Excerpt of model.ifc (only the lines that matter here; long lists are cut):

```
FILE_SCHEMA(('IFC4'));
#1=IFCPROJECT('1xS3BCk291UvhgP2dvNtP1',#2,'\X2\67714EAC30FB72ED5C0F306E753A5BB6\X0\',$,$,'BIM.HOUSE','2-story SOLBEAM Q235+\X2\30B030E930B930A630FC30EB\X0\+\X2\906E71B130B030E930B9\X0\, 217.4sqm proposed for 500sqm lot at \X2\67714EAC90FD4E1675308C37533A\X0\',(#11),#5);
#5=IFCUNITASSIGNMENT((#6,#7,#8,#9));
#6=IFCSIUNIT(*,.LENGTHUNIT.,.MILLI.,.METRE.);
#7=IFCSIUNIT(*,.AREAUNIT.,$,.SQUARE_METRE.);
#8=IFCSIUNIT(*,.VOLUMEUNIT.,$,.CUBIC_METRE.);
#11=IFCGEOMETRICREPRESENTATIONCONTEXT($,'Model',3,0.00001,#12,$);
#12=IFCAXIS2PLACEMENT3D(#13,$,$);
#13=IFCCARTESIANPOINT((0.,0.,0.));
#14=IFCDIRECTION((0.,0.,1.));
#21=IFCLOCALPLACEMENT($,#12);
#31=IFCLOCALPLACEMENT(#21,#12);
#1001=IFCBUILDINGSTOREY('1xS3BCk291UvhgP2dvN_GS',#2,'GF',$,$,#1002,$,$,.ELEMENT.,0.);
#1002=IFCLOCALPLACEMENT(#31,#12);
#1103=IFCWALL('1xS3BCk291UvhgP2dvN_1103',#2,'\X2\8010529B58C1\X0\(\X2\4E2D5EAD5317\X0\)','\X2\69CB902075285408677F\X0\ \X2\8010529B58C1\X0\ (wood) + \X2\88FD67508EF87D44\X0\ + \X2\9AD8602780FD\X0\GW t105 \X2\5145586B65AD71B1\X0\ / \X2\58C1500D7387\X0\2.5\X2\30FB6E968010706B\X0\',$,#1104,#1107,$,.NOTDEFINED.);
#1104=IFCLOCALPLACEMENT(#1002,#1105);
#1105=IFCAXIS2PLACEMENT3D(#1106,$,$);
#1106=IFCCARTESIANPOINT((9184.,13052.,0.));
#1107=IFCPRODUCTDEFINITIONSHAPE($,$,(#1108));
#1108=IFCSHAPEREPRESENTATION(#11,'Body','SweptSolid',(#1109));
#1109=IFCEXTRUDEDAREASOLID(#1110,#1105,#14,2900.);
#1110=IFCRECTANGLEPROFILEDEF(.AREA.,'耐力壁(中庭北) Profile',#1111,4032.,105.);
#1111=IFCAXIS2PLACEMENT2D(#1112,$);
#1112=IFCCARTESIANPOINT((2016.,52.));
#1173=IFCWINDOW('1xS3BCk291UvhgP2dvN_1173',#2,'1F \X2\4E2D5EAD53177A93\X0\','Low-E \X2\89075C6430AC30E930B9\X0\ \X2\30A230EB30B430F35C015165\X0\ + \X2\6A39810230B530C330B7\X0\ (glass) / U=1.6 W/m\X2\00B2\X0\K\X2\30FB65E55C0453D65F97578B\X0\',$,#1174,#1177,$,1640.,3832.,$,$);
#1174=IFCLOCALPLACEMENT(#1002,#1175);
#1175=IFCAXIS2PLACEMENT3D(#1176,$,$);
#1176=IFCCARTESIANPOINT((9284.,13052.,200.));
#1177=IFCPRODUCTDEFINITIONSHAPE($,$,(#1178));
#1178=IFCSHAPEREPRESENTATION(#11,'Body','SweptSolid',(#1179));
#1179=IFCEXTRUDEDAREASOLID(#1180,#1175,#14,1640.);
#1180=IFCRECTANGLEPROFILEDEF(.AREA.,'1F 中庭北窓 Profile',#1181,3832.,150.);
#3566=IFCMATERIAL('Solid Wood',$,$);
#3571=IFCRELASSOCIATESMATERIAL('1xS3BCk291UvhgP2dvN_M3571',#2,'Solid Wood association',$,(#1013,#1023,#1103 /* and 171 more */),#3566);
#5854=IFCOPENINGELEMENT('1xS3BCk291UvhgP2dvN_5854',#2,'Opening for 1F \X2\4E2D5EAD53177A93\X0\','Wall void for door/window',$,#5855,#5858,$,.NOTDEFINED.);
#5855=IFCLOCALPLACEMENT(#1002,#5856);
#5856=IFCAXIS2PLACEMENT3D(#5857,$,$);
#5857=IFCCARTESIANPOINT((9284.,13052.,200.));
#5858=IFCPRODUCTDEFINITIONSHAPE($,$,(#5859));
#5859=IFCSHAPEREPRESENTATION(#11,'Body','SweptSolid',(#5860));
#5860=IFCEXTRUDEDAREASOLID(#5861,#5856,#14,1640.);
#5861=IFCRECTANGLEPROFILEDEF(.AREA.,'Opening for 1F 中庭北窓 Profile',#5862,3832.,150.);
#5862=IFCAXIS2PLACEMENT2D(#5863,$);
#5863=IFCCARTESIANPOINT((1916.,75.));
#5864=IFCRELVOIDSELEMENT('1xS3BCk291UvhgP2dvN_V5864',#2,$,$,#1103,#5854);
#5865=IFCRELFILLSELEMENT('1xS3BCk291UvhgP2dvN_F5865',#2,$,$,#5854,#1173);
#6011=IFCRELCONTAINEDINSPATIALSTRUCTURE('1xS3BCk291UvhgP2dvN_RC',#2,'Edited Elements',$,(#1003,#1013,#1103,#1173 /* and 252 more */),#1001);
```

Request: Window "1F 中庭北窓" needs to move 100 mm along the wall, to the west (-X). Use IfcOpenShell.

```python
import ifcopenshell
import ifcopenshell.api.geometry
import ifcopenshell.util.placement

model = ifcopenshell.open("model.ifc")

window = model.by_id(1173)
opening = window.FillsVoids[0].RelatingOpeningElement
wall = opening.VoidsElements[0].RelatingBuildingElement

wall_matrix = ifcopenshell.util.placement.get_local_placement(wall.ObjectPlacement)
shift = wall_matrix[:3, 0] * -100.0
before = ifcopenshell.util.placement.get_local_placement(window.ObjectPlacement)[:3, 3].copy()

# The window is not placed relative to its opening, so move both.
for product in (opening, window):
    matrix = ifcopenshell.util.placement.get_local_placement(product.ObjectPlacement)
    matrix[:3, 3] += shift
    ifcopenshell.api.geometry.edit_object_placement(model, product=product, matrix=matrix, is_si=False)

after = ifcopenshell.util.placement.get_local_placement(window.ObjectPlacement)[:3, 3]
print("window moved by", (after - before).round(3) + 0.0)

model.write("model_v2.ifc")
```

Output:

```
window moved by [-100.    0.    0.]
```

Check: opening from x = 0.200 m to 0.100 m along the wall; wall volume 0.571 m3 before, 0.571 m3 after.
